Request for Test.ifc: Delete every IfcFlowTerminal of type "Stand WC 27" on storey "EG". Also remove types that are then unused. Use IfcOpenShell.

First a look at what the model holds.

```python
import ifcopenshell
import ifcopenshell.util.element

model = ifcopenshell.open("Test.ifc")
print(model.schema)
storey = next(s for s in model.by_type("IfcBuildingStorey") if s.Name == "EG")
terminals = [e for e in ifcopenshell.util.element.get_decomposition(storey) if e.is_a("IfcFlowTerminal")]
seen = {}
for e in terminals:
    element_type = ifcopenshell.util.element.get_type(e)
    name = element_type.Name if element_type not in (None, e) else None
    seen[name] = seen.get(name, 0) + 1
for name, count in sorted(seen.items(), key=str):
    print(count, "x", name)
```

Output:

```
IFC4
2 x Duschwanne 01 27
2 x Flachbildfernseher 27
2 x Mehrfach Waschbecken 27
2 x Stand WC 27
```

```python
import ifcopenshell
import ifcopenshell.api.root
import ifcopenshell.util.element

model = ifcopenshell.open("Test.ifc")

storey = next(s for s in model.by_type("IfcBuildingStorey") if s.Name == "EG")
terminals = [e for e in ifcopenshell.util.element.get_decomposition(storey) if e.is_a("IfcFlowTerminal")]
targets = [e for e in terminals if (t := ifcopenshell.util.element.get_type(e)) not in (None, e) and t.Name == "Stand WC 27"]
types = {ifcopenshell.util.element.get_type(e) for e in targets} - {None, *targets}

for e in targets:
    ifcopenshell.api.root.remove_product(model, product=e)
print(len(targets), "removed")

unused = [t for t in types if not ifcopenshell.util.element.get_types(t)]
for t in unused:
    ifcopenshell.api.root.remove_product(model, product=t)
print(len(unused), "unused types removed")

model.write("Test-out.ifc")
```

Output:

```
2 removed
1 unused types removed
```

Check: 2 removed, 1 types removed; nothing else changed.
